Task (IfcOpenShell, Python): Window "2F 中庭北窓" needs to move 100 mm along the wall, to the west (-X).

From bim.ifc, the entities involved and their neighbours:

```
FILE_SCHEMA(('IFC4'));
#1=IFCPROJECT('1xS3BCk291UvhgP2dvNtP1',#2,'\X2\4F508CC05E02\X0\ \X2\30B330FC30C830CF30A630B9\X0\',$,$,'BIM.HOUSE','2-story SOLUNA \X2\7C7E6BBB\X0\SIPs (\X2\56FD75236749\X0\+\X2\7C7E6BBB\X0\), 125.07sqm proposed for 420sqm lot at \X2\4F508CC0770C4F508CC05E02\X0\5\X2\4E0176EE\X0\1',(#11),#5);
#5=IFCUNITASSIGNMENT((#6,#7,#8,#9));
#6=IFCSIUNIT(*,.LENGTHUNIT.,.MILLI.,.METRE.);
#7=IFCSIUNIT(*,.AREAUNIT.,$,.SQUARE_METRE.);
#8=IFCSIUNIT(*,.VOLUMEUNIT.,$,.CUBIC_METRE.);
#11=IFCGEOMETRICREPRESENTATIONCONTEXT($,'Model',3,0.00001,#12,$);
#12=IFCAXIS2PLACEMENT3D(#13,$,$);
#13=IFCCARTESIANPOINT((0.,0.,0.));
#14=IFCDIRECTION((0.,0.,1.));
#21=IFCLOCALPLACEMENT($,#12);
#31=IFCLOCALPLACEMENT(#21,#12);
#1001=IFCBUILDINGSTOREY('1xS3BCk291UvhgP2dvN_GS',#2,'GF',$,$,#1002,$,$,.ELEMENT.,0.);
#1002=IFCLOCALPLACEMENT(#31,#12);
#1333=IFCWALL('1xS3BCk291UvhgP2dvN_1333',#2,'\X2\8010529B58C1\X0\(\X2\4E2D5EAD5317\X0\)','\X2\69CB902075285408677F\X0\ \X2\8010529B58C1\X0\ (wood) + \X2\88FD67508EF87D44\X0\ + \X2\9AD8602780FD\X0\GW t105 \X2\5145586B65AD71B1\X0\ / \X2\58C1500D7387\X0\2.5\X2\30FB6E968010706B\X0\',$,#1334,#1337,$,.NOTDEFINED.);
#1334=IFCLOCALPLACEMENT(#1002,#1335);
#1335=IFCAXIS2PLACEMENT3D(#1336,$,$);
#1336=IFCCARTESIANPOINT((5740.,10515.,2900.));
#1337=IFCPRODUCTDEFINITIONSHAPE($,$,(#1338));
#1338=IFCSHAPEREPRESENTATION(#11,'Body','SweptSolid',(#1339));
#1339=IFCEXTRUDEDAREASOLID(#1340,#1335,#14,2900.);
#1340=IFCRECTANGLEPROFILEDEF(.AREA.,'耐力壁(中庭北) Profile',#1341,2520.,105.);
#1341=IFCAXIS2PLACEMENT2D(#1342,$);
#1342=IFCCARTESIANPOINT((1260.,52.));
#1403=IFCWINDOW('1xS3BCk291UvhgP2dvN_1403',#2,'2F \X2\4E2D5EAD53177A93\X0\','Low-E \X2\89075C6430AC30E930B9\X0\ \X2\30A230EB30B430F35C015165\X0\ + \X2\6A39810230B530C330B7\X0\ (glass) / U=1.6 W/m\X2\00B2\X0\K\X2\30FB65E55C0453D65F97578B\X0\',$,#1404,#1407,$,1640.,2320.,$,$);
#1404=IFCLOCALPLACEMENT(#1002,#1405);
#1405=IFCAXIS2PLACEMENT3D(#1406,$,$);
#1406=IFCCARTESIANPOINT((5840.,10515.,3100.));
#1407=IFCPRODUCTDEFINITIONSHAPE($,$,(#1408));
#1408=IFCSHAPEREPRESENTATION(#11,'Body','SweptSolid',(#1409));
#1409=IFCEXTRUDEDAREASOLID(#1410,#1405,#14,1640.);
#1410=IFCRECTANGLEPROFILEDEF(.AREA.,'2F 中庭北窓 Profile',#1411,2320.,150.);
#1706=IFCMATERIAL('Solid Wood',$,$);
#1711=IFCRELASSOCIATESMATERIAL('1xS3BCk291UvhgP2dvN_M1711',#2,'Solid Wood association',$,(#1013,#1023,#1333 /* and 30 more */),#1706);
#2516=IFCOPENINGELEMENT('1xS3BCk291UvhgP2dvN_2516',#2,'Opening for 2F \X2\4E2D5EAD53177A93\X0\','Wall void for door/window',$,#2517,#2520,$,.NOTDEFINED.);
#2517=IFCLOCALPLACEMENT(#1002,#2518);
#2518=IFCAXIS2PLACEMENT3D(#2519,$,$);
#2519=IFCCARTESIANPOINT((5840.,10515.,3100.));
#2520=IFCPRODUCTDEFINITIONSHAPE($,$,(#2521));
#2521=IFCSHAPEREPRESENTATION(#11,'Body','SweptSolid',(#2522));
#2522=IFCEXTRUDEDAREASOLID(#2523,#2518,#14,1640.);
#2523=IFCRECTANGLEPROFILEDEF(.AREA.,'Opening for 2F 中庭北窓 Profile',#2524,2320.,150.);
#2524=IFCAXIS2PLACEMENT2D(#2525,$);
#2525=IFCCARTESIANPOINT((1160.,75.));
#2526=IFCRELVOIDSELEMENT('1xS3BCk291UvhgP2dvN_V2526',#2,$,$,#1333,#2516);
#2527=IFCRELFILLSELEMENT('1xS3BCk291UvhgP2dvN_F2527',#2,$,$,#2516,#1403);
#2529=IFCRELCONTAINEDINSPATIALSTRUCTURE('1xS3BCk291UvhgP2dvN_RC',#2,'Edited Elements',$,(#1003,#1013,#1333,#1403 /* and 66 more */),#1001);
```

```python
import ifcopenshell
import ifcopenshell.api.geometry
import ifcopenshell.util.placement
import ifcopenshell.util.unit

model = ifcopenshell.open("bim.ifc")
unit_scale = ifcopenshell.util.unit.calculate_unit_scale(model)

window = model.by_id(1403)
opening = window.FillsVoids[0].RelatingOpeningElement
wall = opening.VoidsElements[0].RelatingBuildingElement

wall_matrix = ifcopenshell.util.placement.get_local_placement(wall.ObjectPlacement)
shift = wall_matrix[:3, 0] * -0.1 / unit_scale
before = ifcopenshell.util.placement.get_local_placement(window.ObjectPlacement)[:3, 3].copy()

# The window is not placed relative to its opening, so move both.
for product in (opening, window):
    matrix = ifcopenshell.util.placement.get_local_placement(product.ObjectPlacement)
    matrix[:3, 3] += shift
    ifcopenshell.api.geometry.edit_object_placement(model, product=product, matrix=matrix, is_si=False)

after = ifcopenshell.util.placement.get_local_placement(window.ObjectPlacement)[:3, 3]
print("window moved by", (after - before).round(3) + 0.0)

model.write("bim_updated.ifc")
```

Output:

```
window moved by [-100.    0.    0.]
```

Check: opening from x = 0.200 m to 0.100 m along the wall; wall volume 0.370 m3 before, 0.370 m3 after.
